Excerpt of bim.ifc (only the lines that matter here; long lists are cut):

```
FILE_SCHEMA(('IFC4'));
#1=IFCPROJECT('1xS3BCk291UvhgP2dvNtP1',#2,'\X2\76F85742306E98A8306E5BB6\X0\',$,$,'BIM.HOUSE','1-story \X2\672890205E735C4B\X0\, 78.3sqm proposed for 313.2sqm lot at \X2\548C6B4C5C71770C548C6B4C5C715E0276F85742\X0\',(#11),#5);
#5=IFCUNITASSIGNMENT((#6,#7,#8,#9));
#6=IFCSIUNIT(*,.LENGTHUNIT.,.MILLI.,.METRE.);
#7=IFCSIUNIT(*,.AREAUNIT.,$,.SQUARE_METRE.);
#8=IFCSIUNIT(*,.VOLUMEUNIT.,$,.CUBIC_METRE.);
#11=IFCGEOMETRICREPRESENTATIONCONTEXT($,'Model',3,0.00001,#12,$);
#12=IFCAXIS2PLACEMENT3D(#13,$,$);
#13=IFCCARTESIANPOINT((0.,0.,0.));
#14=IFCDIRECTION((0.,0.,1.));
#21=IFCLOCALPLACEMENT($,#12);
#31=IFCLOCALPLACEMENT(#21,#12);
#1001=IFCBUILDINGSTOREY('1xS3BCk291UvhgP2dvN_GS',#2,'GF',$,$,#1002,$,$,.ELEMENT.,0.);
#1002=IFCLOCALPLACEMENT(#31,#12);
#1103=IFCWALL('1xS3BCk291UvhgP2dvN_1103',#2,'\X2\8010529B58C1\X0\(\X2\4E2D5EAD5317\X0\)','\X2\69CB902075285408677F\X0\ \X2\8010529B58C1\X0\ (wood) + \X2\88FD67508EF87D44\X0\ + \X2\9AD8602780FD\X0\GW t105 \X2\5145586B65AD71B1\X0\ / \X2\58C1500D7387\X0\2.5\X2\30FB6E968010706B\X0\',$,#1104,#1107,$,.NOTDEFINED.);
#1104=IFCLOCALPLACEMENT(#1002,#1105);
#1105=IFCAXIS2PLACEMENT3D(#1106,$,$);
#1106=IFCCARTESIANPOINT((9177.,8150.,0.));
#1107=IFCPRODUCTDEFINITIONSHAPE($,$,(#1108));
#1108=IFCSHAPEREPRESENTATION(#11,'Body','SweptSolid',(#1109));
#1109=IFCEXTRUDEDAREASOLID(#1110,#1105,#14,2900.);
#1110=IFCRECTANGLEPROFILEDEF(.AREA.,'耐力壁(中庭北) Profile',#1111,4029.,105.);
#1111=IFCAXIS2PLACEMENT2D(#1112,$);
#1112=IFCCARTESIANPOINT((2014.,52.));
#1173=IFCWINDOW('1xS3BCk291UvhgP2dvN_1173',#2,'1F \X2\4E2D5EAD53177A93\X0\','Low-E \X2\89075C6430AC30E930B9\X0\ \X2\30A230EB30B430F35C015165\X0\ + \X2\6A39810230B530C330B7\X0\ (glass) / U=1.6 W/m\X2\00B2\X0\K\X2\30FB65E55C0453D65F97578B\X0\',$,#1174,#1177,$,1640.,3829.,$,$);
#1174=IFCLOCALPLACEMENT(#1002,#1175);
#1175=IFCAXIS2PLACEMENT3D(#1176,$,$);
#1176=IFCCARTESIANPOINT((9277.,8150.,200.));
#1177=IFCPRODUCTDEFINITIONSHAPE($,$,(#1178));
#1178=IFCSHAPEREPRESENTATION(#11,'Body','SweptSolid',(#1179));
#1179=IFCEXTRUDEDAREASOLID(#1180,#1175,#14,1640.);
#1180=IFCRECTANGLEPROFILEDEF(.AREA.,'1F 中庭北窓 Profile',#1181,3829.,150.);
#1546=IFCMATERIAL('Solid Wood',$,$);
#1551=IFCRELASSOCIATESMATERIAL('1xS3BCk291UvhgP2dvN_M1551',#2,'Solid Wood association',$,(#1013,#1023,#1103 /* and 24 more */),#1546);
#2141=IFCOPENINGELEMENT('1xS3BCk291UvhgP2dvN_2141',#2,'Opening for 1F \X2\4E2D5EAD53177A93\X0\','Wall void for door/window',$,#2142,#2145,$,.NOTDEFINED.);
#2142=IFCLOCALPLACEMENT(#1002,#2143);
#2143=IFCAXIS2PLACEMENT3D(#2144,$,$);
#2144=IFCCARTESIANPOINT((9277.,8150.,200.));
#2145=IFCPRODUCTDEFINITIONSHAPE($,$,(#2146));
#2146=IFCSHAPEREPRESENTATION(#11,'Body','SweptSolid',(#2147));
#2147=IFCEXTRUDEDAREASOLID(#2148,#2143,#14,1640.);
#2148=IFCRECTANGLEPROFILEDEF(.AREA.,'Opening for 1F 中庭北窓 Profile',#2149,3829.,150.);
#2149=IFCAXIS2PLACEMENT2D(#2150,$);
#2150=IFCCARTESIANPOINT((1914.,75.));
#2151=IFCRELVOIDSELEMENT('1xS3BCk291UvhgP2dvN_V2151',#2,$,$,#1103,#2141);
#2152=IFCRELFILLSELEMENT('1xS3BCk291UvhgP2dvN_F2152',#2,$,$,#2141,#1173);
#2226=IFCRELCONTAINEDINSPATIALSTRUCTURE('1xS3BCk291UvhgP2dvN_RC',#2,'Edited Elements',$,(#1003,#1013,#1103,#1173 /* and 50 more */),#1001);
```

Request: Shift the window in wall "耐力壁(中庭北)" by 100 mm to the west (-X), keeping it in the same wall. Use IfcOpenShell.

```python
import ifcopenshell
import ifcopenshell.api.geometry
import ifcopenshell.util.placement

model = ifcopenshell.open("bim.ifc")

window = model.by_guid("1xS3BCk291UvhgP2dvN_1173")
opening = window.FillsVoids[0].RelatingOpeningElement
wall = opening.VoidsElements[0].RelatingBuildingElement

wall_matrix = ifcopenshell.util.placement.get_local_placement(wall.ObjectPlacement)
shift = wall_matrix[:3, 0] * -100.0
before = ifcopenshell.util.placement.get_local_placement(window.ObjectPlacement)[:3, 3].copy()

# The window is not placed relative to its opening, so move both.
for product in (opening, window):
    matrix = ifcopenshell.util.placement.get_local_placement(product.ObjectPlacement)
    matrix[:3, 3] += shift
    ifcopenshell.api.geometry.edit_object_placement(model, product=product, matrix=matrix, is_si=False)

after = ifcopenshell.util.placement.get_local_placement(window.ObjectPlacement)[:3, 3]
print("window moved by", (after - before).round(3) + 0.0)

model.write("bim_v2.ifc")
```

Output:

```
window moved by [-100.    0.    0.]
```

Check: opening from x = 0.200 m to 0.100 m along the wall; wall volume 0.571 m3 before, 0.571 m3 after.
